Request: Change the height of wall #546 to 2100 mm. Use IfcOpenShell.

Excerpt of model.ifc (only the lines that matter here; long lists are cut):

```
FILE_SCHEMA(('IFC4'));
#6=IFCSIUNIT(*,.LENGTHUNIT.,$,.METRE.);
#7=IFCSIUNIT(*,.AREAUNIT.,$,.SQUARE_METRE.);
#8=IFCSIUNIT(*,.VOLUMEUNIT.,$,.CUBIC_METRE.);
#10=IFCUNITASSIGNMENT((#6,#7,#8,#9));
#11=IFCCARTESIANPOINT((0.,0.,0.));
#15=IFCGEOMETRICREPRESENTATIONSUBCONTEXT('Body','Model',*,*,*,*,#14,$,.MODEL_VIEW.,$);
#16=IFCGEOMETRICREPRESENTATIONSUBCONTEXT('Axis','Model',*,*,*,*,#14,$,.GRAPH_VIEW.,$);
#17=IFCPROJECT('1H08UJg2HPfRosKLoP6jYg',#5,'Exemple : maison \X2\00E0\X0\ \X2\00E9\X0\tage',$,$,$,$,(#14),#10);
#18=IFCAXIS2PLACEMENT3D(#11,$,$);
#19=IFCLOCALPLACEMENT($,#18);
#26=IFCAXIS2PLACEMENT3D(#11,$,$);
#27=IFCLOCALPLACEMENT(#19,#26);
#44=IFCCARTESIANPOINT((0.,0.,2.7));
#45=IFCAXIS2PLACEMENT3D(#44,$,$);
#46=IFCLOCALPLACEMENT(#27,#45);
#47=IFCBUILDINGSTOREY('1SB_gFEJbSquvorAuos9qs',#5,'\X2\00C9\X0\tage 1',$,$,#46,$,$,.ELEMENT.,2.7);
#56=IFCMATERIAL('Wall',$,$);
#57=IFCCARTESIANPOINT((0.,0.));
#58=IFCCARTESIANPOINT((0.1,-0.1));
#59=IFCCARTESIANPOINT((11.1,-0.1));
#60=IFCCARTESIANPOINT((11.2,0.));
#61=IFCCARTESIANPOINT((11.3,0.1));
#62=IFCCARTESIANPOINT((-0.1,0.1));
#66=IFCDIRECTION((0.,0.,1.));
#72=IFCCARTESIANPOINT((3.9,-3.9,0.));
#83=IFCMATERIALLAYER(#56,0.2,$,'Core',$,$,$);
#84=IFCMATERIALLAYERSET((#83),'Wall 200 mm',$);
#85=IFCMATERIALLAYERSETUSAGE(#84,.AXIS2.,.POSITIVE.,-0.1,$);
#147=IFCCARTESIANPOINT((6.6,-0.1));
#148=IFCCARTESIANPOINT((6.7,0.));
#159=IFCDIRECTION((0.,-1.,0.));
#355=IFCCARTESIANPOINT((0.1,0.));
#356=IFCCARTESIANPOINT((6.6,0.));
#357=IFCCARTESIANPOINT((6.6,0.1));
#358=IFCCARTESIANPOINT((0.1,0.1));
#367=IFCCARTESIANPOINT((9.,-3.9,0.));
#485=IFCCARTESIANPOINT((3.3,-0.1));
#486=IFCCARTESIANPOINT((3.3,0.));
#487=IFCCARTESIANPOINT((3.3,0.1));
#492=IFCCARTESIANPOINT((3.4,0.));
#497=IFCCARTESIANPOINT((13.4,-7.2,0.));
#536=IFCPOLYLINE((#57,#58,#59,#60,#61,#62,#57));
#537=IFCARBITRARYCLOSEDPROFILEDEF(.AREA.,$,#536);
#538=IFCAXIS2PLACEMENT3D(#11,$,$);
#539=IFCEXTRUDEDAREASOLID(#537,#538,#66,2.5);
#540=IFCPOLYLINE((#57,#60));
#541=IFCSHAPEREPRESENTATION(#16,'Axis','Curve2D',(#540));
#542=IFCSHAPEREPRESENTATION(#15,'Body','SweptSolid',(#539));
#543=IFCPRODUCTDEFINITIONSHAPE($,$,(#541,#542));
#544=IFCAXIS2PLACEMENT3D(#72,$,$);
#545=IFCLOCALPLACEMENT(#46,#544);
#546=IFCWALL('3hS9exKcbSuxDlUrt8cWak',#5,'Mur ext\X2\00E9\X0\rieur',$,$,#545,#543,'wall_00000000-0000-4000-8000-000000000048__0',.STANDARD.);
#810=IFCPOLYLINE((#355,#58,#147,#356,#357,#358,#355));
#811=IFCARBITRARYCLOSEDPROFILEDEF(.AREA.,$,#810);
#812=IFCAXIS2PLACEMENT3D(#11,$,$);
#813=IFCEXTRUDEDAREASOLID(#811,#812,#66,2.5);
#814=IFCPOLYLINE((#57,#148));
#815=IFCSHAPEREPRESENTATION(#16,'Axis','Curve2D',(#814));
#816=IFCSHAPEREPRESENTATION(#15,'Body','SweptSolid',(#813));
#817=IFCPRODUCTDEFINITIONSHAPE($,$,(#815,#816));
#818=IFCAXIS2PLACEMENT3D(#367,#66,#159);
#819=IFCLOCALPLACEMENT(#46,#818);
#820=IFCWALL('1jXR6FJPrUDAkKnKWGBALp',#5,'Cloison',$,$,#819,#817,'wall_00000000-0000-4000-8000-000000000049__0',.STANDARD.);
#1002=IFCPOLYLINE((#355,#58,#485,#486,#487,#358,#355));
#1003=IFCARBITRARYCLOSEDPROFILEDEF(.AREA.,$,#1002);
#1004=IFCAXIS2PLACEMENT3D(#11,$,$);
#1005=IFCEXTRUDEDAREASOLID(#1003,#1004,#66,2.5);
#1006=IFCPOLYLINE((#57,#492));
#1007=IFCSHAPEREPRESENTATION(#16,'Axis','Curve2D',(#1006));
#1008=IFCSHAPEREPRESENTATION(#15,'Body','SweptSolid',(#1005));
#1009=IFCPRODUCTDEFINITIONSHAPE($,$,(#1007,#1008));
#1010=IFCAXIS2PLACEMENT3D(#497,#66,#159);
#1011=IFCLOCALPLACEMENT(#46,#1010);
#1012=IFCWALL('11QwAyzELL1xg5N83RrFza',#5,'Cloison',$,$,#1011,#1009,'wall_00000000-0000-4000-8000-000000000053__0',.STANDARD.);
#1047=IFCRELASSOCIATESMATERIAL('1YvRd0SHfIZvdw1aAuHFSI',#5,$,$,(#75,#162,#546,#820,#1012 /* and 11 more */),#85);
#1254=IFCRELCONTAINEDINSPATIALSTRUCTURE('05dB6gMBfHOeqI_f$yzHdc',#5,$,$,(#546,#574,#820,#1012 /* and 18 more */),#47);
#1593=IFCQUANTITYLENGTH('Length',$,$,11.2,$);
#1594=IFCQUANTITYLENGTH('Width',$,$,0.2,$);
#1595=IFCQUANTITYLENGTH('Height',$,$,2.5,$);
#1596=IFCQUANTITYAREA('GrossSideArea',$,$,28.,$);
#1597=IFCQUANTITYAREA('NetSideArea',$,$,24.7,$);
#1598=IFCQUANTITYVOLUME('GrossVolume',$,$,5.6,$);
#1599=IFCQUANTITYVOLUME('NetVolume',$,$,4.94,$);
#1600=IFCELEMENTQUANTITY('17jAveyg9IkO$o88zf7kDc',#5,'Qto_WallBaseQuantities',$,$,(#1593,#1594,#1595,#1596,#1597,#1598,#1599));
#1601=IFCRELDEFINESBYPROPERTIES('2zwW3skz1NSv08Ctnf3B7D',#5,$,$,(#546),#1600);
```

```python
import ifcopenshell
import ifcopenshell.api.pset
import ifcopenshell.geom
import ifcopenshell.util.element
import ifcopenshell.util.representation
import ifcopenshell.util.shape
import ifcopenshell.util.unit

model = ifcopenshell.open("model.ifc")
unit_scale = ifcopenshell.util.unit.calculate_unit_scale(model)
area_scale = ifcopenshell.util.unit.calculate_unit_scale(model, "AREAUNIT")
volume_scale = ifcopenshell.util.unit.calculate_unit_scale(model, "VOLUMEUNIT")
settings = ifcopenshell.geom.settings()


def volume(element):
    """Net volume in cubic metres, openings subtracted."""
    shape = ifcopenshell.geom.create_shape(settings, element)
    return ifcopenshell.util.shape.get_volume(shape.geometry)


wall = model.by_id(546)
before = volume(wall)

body = ifcopenshell.util.representation.get_representation(wall, "Model", "Body")
solid = body.Items[0]
old_height = solid.Depth
solid.Depth = 2.1 / unit_scale
after = volume(wall)
thickness = 0.2  # wall thickness in metres

# Update the stored height, areas and volumes.
qto = model.by_id(ifcopenshell.util.element.get_pset(wall, "Qto_WallBaseQuantities", should_inherit=False)["id"])
ifcopenshell.api.pset.edit_qto(model, qto=qto, properties={
    "Height": solid.Depth,
    "GrossSideArea": ifcopenshell.util.element.get_pset(wall, "Qto_WallBaseQuantities", "GrossSideArea") * solid.Depth / old_height,
    "NetSideArea": after / thickness / area_scale,
    "GrossVolume": ifcopenshell.util.element.get_pset(wall, "Qto_WallBaseQuantities", "GrossVolume") * solid.Depth / old_height,
    "NetVolume": after / volume_scale,
})

print(f"height {old_height:g} -> {solid.Depth:g}, volume {before:.3f} -> {after:.3f} m3")

model.write("model_v2.ifc")
```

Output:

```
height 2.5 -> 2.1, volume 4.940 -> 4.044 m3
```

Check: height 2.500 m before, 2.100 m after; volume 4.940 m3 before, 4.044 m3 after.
